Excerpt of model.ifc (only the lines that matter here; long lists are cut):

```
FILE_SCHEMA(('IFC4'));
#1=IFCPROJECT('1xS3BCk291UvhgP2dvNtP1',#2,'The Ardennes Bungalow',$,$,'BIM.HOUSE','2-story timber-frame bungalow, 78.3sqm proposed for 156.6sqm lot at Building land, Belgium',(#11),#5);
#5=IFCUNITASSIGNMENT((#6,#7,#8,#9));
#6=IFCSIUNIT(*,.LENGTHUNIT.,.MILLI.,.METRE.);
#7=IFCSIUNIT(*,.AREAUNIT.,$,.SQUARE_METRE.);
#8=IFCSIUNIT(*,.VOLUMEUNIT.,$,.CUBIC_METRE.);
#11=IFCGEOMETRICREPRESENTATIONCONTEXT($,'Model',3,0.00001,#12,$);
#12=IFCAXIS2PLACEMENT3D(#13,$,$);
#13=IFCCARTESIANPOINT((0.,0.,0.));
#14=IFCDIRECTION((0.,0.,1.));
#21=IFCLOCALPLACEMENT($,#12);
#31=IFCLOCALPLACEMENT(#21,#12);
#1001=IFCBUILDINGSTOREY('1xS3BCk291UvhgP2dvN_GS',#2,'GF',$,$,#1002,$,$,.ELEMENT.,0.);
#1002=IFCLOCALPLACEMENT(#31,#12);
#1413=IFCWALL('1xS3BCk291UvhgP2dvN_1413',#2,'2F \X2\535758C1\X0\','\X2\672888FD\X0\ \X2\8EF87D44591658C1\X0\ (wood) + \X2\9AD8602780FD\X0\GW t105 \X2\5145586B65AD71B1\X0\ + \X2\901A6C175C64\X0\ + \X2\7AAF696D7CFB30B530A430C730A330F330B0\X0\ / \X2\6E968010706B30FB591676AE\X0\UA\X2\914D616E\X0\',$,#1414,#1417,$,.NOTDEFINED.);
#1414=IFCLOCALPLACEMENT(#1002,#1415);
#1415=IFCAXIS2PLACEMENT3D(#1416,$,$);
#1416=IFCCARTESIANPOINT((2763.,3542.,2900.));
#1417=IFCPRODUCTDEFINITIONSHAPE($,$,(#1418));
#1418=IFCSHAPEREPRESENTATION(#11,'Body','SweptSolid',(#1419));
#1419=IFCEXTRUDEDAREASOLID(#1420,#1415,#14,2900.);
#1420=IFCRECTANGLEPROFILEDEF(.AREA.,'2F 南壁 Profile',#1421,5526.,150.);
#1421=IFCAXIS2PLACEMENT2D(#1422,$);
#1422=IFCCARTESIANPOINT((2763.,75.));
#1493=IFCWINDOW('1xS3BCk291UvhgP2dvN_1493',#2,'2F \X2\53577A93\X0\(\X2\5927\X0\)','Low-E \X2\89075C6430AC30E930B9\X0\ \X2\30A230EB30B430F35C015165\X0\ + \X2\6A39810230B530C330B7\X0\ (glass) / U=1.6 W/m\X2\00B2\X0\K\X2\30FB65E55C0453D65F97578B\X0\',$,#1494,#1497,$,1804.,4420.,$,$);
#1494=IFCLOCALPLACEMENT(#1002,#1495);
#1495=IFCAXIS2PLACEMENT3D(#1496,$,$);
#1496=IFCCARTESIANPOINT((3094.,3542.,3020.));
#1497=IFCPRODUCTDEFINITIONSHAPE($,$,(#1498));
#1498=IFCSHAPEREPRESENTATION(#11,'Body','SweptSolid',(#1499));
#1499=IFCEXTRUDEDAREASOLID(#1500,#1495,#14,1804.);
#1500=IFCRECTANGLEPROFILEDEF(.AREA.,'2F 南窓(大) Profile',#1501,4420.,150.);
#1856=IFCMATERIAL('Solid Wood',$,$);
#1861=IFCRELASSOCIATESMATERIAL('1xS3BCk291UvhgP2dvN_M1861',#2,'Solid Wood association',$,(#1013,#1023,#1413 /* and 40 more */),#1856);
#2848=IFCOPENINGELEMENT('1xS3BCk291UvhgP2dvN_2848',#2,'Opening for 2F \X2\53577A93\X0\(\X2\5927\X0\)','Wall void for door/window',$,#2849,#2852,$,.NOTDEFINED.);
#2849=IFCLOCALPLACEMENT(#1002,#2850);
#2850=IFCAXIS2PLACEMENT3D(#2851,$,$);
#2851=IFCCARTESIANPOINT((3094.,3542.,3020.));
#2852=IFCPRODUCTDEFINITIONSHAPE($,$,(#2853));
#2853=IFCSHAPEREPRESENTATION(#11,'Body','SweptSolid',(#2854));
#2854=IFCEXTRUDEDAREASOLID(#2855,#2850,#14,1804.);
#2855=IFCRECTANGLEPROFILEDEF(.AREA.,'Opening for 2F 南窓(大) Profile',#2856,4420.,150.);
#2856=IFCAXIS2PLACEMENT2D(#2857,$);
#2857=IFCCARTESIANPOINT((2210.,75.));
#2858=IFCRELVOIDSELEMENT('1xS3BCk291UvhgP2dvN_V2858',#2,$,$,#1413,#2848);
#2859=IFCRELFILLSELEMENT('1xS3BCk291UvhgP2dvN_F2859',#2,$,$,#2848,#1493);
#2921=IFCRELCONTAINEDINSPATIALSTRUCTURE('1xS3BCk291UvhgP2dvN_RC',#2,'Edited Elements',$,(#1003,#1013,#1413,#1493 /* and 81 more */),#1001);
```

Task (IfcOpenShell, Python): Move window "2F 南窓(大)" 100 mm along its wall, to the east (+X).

```python
import ifcopenshell
import ifcopenshell.api.geometry
import ifcopenshell.util.placement
import ifcopenshell.util.unit

model = ifcopenshell.open("model.ifc")
unit_scale = ifcopenshell.util.unit.calculate_unit_scale(model)

window = model.by_guid("1xS3BCk291UvhgP2dvN_1493")
opening = window.FillsVoids[0].RelatingOpeningElement
wall = opening.VoidsElements[0].RelatingBuildingElement

wall_matrix = ifcopenshell.util.placement.get_local_placement(wall.ObjectPlacement)
shift = wall_matrix[:3, 0] * 0.1 / unit_scale
before = ifcopenshell.util.placement.get_local_placement(window.ObjectPlacement)[:3, 3].copy()

# The window is not placed relative to its opening, so move both.
for product in (opening, window):
    matrix = ifcopenshell.util.placement.get_local_placement(product.ObjectPlacement)
    matrix[:3, 3] += shift
    ifcopenshell.api.geometry.edit_object_placement(model, product=product, matrix=matrix, is_si=False)

after = ifcopenshell.util.placement.get_local_placement(window.ObjectPlacement)[:3, 3]
print("window moved by", (after - before).round(3) + 0.0)

model.write("model_edited.ifc")
```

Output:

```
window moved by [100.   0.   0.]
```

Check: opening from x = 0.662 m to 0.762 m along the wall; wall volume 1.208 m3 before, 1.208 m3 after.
